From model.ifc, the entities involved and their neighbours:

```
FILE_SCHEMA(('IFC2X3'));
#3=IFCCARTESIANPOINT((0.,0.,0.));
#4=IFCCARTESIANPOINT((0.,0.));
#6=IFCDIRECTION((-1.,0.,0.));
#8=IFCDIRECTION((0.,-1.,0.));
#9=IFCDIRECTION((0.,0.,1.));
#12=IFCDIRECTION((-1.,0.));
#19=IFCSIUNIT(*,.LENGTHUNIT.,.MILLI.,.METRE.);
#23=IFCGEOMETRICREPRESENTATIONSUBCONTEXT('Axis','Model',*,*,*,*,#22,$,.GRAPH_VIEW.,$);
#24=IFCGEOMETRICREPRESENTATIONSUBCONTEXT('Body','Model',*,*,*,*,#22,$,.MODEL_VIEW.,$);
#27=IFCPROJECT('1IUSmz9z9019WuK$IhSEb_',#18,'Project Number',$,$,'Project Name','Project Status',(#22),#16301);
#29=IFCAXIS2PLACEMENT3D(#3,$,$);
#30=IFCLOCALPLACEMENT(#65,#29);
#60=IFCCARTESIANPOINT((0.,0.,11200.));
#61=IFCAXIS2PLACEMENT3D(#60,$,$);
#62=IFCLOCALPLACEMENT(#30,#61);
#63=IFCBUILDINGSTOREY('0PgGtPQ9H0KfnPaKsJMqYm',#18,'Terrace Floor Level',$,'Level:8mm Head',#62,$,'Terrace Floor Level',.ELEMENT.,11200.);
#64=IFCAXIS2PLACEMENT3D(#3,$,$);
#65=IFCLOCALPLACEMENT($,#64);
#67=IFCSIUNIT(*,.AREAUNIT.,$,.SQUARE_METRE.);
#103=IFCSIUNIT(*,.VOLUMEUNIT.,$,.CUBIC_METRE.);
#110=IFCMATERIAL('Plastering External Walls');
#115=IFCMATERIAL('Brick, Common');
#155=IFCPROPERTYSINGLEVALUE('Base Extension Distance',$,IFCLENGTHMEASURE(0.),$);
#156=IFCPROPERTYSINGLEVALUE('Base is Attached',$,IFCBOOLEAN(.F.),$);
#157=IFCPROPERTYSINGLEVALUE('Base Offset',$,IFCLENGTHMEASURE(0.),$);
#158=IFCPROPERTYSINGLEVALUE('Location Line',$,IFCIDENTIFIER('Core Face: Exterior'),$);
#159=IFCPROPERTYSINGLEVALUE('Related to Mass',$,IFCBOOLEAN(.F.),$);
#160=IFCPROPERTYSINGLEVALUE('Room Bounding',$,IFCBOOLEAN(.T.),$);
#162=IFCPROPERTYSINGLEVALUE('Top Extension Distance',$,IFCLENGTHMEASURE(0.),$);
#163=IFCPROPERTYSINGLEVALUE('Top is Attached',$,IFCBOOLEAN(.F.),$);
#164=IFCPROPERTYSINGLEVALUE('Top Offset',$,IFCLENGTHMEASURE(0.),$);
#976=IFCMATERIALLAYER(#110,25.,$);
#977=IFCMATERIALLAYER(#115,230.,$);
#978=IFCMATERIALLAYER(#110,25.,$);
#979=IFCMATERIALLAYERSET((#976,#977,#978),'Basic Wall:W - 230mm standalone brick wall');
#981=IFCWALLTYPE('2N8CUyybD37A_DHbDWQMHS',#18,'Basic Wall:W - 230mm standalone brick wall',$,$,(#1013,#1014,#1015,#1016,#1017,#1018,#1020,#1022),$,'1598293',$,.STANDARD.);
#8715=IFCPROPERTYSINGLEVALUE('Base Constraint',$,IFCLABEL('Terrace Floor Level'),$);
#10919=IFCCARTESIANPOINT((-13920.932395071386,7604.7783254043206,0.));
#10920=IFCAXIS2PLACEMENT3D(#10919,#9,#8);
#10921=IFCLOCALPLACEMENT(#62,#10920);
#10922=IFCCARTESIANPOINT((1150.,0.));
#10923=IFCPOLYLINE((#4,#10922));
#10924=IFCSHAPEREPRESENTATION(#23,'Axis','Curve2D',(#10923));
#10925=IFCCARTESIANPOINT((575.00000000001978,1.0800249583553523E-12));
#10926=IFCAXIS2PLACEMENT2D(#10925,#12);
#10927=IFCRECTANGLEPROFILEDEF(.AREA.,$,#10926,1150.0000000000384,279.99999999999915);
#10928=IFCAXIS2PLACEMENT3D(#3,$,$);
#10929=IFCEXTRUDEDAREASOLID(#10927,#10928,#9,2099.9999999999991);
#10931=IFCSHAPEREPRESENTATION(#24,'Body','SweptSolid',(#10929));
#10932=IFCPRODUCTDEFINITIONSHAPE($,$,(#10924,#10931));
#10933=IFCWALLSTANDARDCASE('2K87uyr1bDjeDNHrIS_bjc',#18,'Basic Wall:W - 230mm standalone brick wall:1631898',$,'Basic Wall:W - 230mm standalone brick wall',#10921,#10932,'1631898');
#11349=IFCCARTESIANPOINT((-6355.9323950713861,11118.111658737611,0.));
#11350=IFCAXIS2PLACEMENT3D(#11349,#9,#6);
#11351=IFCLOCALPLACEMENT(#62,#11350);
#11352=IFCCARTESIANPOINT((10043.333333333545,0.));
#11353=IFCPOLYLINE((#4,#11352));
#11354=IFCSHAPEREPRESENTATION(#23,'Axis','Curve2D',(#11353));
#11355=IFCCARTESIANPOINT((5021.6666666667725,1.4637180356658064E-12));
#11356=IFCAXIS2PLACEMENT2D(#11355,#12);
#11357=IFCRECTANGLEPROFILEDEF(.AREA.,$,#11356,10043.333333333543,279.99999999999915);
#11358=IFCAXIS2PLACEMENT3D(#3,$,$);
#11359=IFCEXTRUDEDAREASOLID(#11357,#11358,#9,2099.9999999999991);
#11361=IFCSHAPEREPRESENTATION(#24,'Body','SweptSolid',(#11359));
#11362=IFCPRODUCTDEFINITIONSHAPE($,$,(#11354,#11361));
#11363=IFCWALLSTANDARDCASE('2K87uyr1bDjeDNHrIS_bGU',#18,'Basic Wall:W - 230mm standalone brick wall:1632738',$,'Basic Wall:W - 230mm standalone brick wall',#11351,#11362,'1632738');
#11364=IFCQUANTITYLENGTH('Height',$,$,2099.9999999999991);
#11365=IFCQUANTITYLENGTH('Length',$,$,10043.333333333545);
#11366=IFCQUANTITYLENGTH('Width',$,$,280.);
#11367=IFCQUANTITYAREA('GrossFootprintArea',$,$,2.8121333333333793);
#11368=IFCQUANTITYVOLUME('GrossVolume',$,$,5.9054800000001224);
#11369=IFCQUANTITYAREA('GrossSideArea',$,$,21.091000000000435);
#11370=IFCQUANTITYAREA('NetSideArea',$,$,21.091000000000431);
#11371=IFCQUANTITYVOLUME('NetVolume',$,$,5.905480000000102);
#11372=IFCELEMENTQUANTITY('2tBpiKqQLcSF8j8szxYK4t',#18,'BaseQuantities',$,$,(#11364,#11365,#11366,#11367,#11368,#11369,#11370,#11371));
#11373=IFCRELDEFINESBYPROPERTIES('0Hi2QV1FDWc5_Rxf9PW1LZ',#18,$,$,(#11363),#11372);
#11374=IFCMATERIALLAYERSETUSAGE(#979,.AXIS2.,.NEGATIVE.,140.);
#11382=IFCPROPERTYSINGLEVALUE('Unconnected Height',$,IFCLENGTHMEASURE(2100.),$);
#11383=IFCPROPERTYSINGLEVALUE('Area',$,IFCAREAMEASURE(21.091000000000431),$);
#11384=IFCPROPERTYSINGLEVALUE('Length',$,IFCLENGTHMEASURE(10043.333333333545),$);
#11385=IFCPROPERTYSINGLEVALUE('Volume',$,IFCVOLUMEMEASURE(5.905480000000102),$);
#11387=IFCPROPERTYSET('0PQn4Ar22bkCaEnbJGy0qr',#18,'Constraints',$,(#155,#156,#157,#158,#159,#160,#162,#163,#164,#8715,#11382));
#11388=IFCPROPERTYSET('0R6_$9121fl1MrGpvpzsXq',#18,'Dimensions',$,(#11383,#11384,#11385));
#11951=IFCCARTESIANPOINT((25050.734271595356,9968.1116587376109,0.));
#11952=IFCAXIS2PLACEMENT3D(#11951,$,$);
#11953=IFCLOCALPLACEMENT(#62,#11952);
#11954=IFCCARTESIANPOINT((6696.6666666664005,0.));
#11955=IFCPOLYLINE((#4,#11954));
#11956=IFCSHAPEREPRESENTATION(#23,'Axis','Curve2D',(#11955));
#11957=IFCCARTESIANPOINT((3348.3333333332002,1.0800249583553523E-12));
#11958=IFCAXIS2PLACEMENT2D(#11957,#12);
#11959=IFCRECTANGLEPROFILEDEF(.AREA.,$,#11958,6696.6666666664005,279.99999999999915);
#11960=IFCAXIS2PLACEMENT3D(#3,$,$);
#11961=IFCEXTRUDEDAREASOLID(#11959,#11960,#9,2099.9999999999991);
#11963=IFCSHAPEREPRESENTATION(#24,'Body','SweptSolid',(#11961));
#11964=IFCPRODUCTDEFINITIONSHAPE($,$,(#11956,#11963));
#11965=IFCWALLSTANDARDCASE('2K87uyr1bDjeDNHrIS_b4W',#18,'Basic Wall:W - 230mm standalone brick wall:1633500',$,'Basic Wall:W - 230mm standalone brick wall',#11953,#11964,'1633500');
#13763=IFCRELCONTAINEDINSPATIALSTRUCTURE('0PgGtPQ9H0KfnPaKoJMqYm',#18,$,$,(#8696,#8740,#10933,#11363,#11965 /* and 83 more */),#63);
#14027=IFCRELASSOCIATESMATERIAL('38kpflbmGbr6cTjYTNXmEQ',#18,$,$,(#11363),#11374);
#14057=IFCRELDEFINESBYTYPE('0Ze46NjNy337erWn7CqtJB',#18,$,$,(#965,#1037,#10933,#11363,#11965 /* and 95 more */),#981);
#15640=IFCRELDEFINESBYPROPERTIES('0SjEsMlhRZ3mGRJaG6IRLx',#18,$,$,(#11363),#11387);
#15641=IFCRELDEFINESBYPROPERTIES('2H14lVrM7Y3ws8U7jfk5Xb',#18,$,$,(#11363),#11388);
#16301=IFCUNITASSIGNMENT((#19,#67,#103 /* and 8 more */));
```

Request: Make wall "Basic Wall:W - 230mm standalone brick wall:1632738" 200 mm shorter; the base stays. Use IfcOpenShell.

```python
import ifcopenshell
import ifcopenshell.api.pset
import ifcopenshell.geom
import ifcopenshell.util.element
import ifcopenshell.util.representation
import ifcopenshell.util.shape
import ifcopenshell.util.unit

model = ifcopenshell.open("model.ifc")
unit_scale = ifcopenshell.util.unit.calculate_unit_scale(model)
area_scale = ifcopenshell.util.unit.calculate_unit_scale(model, "AREAUNIT")
volume_scale = ifcopenshell.util.unit.calculate_unit_scale(model, "VOLUMEUNIT")
settings = ifcopenshell.geom.settings()


def volume(element):
    """Net volume in cubic metres, openings subtracted."""
    shape = ifcopenshell.geom.create_shape(settings, element)
    return ifcopenshell.util.shape.get_volume(shape.geometry)


wall = model.by_guid("2K87uyr1bDjeDNHrIS_bGU")
before = volume(wall)

body = ifcopenshell.util.representation.get_representation(wall, "Model", "Body")
solid = body.Items[0]
old_height = solid.Depth
solid.Depth -= 0.2 / unit_scale
after = volume(wall)
thickness = 0.28  # wall thickness in metres

# Update the stored height, areas and volumes.
qto = model.by_id(ifcopenshell.util.element.get_pset(wall, "BaseQuantities", should_inherit=False)["id"])
ifcopenshell.api.pset.edit_qto(model, qto=qto, properties={
    "Height": solid.Depth,
    "GrossVolume": ifcopenshell.util.element.get_pset(wall, "BaseQuantities", "GrossVolume") * solid.Depth / old_height,
    "GrossSideArea": ifcopenshell.util.element.get_pset(wall, "BaseQuantities", "GrossSideArea") * solid.Depth / old_height,
    "NetSideArea": after / thickness / area_scale,
    "NetVolume": after / volume_scale,
})
pset = model.by_id(ifcopenshell.util.element.get_pset(wall, "Constraints", should_inherit=False)["id"])
ifcopenshell.api.pset.edit_pset(model, pset=pset, properties={
    "Unconnected Height": model.create_entity("IfcLengthMeasure", solid.Depth),
})
pset = model.by_id(ifcopenshell.util.element.get_pset(wall, "Dimensions", should_inherit=False)["id"])
ifcopenshell.api.pset.edit_pset(model, pset=pset, properties={
    "Area": model.create_entity("IfcAreaMeasure", after / thickness / area_scale),
    "Volume": model.create_entity("IfcVolumeMeasure", after / volume_scale),
})

print(f"height {old_height:g} -> {solid.Depth:g}, volume {before:.3f} -> {after:.3f} m3")

model.write("model-out.ifc")
```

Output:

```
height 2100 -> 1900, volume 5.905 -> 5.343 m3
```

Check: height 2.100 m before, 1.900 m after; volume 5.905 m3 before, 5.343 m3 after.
